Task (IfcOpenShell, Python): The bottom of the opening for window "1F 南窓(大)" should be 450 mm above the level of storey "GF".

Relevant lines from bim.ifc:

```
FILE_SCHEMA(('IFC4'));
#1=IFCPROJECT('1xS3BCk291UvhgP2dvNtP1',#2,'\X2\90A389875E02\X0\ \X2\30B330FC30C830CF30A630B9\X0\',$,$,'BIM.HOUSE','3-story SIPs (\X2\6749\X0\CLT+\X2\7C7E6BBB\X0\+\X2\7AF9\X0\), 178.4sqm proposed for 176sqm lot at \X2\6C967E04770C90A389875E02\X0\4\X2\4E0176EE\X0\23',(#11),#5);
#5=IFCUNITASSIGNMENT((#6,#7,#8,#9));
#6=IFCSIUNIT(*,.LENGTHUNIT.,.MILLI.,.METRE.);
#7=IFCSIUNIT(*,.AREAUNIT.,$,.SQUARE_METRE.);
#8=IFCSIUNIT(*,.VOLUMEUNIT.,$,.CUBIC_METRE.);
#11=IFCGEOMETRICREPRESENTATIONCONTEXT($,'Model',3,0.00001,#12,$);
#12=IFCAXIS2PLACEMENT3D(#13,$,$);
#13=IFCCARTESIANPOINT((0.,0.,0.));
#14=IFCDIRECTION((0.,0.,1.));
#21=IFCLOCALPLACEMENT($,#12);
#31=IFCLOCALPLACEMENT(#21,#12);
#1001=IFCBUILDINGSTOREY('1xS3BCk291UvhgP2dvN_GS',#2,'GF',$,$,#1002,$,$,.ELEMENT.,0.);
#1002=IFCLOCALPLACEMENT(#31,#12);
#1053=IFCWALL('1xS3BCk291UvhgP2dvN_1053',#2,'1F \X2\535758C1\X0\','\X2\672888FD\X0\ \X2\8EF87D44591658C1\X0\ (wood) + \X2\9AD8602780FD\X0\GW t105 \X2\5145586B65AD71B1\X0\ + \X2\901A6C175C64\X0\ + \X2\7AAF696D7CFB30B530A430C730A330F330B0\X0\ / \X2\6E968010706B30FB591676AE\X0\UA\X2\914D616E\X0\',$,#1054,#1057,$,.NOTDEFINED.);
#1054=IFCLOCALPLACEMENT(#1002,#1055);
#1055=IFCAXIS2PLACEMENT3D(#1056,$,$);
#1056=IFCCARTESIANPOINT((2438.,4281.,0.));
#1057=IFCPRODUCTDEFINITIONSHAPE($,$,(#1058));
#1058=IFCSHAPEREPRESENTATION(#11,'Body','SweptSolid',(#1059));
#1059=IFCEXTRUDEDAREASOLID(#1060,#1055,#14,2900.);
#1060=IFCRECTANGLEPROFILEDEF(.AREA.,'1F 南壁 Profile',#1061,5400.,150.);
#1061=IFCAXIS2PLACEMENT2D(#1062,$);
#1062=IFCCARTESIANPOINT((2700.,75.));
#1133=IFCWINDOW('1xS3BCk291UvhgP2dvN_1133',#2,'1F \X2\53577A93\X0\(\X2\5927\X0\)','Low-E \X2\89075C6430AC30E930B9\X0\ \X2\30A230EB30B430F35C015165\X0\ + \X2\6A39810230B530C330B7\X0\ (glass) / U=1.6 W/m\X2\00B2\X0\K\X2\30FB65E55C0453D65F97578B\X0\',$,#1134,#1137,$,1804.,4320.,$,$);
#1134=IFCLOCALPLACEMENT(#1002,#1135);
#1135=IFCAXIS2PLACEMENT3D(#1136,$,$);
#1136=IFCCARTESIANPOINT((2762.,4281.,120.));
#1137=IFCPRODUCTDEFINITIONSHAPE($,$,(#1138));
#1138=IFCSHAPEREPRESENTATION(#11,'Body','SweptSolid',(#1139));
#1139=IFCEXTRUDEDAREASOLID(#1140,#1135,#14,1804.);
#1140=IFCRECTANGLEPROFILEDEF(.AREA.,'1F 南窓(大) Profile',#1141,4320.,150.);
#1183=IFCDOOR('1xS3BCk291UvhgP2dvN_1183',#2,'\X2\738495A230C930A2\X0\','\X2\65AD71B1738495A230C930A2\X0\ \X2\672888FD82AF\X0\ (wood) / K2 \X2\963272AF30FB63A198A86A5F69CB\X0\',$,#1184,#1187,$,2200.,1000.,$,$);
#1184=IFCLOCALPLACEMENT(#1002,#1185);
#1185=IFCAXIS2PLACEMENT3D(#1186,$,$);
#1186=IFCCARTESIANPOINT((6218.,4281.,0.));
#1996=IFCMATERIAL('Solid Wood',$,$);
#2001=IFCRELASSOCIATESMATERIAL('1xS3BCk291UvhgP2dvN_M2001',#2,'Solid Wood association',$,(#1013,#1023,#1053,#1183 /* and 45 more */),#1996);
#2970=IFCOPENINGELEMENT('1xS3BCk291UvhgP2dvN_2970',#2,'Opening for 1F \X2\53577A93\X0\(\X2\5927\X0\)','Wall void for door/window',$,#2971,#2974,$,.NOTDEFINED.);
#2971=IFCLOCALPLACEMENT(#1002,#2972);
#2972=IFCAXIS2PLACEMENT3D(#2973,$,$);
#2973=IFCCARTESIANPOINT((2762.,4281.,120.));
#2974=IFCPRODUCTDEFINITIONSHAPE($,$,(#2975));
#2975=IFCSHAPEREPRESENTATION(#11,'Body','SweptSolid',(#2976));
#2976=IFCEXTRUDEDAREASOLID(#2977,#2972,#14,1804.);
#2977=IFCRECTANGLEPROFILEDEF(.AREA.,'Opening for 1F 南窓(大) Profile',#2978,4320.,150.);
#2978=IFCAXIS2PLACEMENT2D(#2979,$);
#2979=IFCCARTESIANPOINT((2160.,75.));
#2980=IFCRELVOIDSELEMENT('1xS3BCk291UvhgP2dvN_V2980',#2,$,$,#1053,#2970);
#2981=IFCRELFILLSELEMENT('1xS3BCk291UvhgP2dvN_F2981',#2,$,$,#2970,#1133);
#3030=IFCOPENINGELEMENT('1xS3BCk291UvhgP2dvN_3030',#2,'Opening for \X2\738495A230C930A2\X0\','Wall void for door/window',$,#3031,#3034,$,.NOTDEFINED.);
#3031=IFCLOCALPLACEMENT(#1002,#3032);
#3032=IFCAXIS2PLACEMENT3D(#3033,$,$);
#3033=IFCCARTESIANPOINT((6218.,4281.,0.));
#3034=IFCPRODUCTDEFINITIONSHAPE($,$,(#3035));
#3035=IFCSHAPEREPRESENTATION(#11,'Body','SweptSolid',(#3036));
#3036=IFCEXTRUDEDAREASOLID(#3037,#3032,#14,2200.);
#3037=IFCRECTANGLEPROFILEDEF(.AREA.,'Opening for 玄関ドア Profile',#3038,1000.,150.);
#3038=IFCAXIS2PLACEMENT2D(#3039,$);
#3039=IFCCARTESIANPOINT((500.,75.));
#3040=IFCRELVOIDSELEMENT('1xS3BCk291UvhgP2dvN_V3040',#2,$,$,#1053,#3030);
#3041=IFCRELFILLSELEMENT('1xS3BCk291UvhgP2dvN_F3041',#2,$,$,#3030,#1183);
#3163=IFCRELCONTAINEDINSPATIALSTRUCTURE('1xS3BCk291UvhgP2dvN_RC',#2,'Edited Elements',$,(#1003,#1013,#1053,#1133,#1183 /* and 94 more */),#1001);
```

```python
import numpy as np
import ifcopenshell
import ifcopenshell.api.geometry
import ifcopenshell.geom
import ifcopenshell.util.element
import ifcopenshell.util.placement
import ifcopenshell.util.shape
import ifcopenshell.util.unit

model = ifcopenshell.open("bim.ifc")
unit_scale = ifcopenshell.util.unit.calculate_unit_scale(model)

window = model.by_id(1133)
opening = window.FillsVoids[0].RelatingOpeningElement
storey = ifcopenshell.util.element.get_container(window, ifc_class="IfcBuildingStorey")
level = ifcopenshell.util.placement.get_local_placement(storey.ObjectPlacement)[2, 3]

# The opening's origin need not be at the sill, so measure its lowest point.
shape = ifcopenshell.geom.create_shape(ifcopenshell.geom.settings(), opening)
bottom = ifcopenshell.util.shape.get_shape_bottom_elevation(shape, shape.geometry) / unit_scale
dz = level + 0.45 / unit_scale - bottom

shift = np.array([0.0, 0.0, dz])
# The window is not placed relative to its opening, so move both.
for product in (opening, window):
    matrix = ifcopenshell.util.placement.get_local_placement(product.ObjectPlacement)
    matrix[:3, 3] += shift
    ifcopenshell.api.geometry.edit_object_placement(model, product=product, matrix=matrix, is_si=False)

print(f"moved by {dz * unit_scale:+.3f} m")

model.write("bim_updated.ifc")
```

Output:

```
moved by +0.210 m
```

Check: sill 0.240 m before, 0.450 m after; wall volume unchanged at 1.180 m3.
